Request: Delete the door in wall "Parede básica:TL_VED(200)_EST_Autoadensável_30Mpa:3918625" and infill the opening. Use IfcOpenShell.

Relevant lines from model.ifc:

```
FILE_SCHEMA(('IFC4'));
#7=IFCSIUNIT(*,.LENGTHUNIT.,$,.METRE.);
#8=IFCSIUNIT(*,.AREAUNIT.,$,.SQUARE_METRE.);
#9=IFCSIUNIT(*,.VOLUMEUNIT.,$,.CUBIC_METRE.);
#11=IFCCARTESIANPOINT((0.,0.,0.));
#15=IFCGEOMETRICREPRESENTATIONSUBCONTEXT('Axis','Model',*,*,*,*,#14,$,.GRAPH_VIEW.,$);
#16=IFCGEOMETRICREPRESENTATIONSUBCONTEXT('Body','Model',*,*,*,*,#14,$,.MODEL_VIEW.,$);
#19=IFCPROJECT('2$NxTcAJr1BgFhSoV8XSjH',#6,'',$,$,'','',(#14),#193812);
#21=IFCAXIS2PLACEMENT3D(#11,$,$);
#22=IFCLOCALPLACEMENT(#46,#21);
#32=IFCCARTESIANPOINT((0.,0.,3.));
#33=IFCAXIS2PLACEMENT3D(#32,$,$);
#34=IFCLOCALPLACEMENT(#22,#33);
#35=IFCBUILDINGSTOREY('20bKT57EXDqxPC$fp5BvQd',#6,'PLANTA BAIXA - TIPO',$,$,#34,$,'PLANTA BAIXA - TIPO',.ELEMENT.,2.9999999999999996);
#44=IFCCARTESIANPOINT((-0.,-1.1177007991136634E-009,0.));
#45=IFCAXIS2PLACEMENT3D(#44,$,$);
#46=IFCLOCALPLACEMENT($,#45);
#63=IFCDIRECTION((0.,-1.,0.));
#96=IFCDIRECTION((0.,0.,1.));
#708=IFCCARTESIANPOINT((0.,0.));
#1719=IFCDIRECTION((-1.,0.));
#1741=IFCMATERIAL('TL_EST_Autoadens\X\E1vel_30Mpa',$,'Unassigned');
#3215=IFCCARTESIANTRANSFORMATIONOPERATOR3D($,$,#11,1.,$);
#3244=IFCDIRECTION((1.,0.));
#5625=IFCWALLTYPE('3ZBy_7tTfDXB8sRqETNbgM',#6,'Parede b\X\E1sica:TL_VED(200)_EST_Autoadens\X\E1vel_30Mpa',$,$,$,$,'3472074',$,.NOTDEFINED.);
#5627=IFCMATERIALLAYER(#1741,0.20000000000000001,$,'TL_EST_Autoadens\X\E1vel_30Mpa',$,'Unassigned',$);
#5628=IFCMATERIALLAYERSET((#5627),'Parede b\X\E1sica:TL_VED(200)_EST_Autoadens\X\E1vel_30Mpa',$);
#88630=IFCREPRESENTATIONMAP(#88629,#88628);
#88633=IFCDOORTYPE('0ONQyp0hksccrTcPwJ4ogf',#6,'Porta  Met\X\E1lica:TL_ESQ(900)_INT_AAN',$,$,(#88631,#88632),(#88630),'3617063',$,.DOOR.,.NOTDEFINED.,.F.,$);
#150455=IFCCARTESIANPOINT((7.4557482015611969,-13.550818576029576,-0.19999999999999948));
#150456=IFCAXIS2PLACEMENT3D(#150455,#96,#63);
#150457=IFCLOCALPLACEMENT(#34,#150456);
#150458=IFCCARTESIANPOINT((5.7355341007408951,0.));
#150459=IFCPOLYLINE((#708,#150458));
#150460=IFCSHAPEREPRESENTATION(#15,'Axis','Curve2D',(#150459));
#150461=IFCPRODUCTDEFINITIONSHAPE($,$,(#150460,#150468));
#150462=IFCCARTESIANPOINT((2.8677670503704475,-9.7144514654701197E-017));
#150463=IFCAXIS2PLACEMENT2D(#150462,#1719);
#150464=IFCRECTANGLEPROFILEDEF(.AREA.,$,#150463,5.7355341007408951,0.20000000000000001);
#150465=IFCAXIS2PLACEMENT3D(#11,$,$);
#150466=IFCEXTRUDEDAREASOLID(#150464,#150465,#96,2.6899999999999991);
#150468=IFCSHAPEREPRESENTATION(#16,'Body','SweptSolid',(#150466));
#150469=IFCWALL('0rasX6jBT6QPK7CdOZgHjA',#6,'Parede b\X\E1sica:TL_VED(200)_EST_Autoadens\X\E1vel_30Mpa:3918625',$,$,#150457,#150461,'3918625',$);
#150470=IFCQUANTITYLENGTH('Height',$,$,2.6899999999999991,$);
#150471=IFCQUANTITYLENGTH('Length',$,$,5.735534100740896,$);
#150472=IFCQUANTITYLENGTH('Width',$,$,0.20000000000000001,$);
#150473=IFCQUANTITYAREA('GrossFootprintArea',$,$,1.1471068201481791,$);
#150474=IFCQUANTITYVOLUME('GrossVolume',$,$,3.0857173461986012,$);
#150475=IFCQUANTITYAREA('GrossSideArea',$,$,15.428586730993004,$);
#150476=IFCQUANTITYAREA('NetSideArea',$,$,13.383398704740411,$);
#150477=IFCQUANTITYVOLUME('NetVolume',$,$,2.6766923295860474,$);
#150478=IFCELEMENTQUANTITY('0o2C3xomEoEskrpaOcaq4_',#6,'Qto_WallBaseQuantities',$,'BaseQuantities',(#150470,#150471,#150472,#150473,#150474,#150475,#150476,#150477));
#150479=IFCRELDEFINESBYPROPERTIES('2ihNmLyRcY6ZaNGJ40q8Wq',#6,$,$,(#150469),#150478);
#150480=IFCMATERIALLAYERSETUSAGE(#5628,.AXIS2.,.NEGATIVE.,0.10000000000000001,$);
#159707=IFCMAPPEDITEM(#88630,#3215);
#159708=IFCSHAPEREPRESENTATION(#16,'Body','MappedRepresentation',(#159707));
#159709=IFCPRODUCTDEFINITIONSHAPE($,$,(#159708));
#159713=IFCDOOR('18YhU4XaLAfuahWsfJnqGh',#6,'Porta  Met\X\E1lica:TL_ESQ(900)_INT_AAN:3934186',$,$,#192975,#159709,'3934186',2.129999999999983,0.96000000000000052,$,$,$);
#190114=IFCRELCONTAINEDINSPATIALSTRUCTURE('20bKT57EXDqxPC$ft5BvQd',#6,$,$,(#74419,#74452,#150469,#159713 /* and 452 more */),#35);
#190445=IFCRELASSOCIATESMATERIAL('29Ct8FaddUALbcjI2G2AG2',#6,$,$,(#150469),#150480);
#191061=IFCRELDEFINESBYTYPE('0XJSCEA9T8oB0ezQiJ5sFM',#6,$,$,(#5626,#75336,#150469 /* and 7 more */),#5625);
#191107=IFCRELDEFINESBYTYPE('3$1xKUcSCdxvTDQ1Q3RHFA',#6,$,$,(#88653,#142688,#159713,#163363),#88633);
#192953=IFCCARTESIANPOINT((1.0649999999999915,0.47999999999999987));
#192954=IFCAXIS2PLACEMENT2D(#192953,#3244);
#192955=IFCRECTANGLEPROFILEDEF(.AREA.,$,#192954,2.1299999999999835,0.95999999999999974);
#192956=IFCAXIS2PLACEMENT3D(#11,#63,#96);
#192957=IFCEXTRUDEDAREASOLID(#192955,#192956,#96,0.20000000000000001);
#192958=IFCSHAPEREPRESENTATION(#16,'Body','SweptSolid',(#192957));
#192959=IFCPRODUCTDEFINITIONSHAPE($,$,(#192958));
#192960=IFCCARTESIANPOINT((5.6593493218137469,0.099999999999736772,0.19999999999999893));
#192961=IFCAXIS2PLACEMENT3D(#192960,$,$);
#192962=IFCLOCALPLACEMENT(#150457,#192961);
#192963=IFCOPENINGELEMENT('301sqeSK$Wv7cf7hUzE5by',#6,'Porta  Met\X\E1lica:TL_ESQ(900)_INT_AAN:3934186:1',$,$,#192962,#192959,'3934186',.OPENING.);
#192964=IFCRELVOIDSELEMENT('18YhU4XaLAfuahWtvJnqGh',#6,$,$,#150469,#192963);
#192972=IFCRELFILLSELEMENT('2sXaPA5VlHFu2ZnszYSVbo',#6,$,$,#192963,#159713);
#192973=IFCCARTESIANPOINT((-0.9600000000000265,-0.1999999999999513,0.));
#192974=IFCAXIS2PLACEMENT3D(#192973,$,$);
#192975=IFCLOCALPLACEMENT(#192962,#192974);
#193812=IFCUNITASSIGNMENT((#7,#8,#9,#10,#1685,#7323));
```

```python
import ifcopenshell
import ifcopenshell.api.feature
import ifcopenshell.api.pset
import ifcopenshell.api.root
import ifcopenshell.geom
import ifcopenshell.util.element
import ifcopenshell.util.shape
import ifcopenshell.util.unit

model = ifcopenshell.open("model.ifc")
area_scale = ifcopenshell.util.unit.calculate_unit_scale(model, "AREAUNIT")
volume_scale = ifcopenshell.util.unit.calculate_unit_scale(model, "VOLUMEUNIT")
settings = ifcopenshell.geom.settings()


def volume(element):
    """Net volume in cubic metres, openings subtracted."""
    shape = ifcopenshell.geom.create_shape(settings, element)
    return ifcopenshell.util.shape.get_volume(shape.geometry)


door = model.by_guid("18YhU4XaLAfuahWsfJnqGh")
opening = door.FillsVoids[0].RelatingOpeningElement
wall = opening.VoidsElements[0].RelatingBuildingElement
before = volume(wall)

ifcopenshell.api.root.remove_product(model, product=door)
ifcopenshell.api.feature.remove_feature(model, feature=opening)

after = volume(wall)
thickness = 0.2  # wall thickness in metres

# Update the wall's stored quantities.
qto = model.by_id(ifcopenshell.util.element.get_pset(wall, "Qto_WallBaseQuantities", should_inherit=False)["id"])
ifcopenshell.api.pset.edit_qto(model, qto=qto, properties={
    "NetSideArea": after / thickness / area_scale,
    "NetVolume": after / volume_scale,
})

print(f"wall volume {before:.3f} -> {after:.3f} m3")

model.write("model-out.ifc")
```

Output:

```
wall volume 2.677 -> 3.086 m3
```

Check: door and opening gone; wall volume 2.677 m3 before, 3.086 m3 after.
